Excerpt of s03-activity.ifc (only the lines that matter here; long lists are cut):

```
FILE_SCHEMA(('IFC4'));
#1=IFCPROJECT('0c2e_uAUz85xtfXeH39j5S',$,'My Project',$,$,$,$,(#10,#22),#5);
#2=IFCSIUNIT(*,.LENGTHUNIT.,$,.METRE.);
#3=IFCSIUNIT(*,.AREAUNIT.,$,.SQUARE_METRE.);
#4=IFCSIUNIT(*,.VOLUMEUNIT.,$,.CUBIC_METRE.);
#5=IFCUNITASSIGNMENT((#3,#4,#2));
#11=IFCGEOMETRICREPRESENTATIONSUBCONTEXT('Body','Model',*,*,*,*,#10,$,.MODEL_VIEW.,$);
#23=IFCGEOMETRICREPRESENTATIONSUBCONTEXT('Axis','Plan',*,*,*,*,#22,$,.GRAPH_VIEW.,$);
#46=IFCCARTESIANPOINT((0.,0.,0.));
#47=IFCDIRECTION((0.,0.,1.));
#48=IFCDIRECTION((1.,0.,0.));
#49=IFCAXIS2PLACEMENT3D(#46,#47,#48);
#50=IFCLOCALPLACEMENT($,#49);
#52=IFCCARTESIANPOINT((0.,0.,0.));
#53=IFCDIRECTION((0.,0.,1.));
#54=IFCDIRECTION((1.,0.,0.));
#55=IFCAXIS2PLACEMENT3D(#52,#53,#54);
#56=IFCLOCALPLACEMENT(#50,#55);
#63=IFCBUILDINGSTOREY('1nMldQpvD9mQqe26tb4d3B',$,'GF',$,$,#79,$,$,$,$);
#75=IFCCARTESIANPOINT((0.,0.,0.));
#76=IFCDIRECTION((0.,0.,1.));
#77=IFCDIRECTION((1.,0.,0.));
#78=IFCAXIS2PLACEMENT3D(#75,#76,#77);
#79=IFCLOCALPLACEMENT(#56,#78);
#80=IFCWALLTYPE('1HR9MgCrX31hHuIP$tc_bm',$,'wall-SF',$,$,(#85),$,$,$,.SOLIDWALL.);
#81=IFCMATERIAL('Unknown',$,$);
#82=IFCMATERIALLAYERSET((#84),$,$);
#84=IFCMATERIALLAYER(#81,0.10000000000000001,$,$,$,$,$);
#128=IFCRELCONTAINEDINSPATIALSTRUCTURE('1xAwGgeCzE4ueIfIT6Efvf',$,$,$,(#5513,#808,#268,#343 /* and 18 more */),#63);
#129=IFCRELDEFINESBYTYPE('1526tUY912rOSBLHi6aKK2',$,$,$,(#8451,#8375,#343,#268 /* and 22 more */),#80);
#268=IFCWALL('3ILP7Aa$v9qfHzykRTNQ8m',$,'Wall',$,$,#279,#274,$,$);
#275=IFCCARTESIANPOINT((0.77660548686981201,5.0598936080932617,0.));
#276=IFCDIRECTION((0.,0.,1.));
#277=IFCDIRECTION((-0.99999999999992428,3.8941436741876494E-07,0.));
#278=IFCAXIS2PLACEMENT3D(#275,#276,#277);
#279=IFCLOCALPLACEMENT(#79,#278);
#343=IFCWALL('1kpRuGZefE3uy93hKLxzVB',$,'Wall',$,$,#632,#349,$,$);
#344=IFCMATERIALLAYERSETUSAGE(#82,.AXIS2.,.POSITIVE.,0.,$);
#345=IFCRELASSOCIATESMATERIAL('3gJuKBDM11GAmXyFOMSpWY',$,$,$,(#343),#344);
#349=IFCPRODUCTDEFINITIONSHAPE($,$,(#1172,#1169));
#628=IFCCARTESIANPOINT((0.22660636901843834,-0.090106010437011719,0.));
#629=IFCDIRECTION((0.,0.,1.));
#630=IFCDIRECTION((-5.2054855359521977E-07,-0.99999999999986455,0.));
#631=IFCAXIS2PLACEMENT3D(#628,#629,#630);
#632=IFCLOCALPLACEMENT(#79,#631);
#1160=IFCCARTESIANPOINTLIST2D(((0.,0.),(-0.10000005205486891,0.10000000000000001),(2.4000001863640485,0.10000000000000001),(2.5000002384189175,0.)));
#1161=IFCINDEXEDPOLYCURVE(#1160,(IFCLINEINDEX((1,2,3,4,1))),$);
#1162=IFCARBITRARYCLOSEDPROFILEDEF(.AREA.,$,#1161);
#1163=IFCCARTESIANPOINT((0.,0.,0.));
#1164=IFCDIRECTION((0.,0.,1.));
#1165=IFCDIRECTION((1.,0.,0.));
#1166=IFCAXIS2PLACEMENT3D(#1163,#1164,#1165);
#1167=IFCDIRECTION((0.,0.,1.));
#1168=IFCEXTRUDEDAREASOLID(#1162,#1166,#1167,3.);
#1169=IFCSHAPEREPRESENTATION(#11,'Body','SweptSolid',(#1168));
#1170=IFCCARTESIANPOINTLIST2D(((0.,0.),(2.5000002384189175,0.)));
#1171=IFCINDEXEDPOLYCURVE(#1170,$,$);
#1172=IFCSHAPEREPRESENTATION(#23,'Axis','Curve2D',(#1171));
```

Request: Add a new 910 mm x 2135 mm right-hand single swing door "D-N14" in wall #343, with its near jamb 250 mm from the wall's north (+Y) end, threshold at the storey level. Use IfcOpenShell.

```python
import numpy as np
import ifcopenshell
import ifcopenshell.api.feature
import ifcopenshell.api.geometry
import ifcopenshell.api.root
import ifcopenshell.api.spatial
import ifcopenshell.geom
import ifcopenshell.util.element
import ifcopenshell.util.placement
import ifcopenshell.util.representation
import ifcopenshell.util.shape
import ifcopenshell.util.unit

model = ifcopenshell.open("s03-activity.ifc")
unit_scale = ifcopenshell.util.unit.calculate_unit_scale(model)
settings = ifcopenshell.geom.settings()


def volume(element):
    """Net volume in cubic metres, openings subtracted."""
    shape = ifcopenshell.geom.create_shape(settings, element)
    return ifcopenshell.util.shape.get_volume(shape.geometry)


wall = model.by_guid("1kpRuGZefE3uy93hKLxzVB")
storey = ifcopenshell.util.element.get_container(wall, ifc_class="IfcBuildingStorey")
context = ifcopenshell.util.representation.get_context(model, "Model", "Body", "MODEL_VIEW")
before = volume(wall)

width, height, from_end, sill = 0.91, 2.135, 0.25, 0.0  # metres

# The wall runs along its own X axis, and the end named is its -X end.
wall_shape = ifcopenshell.geom.create_shape(settings, wall)
x, y, z = ifcopenshell.util.shape.get_vertices(wall_shape.geometry).T
start = x.min() + from_end
face, thickness = float(y.min()), float(y.max() - y.min())
wall_matrix = ifcopenshell.util.placement.get_local_placement(wall.ObjectPlacement)
level = ifcopenshell.util.placement.get_local_placement(storey.ObjectPlacement)[2, 3]


def in_wall(x, y):
    """Placement at x, y metres in the wall's axes, at sill height."""
    matrix = wall_matrix.copy()
    matrix[:, 3] = wall_matrix @ np.array([x / unit_scale, y / unit_scale, 0.0, 1.0])
    matrix[2, 3] = level + sill / unit_scale
    return matrix


# Opening: a box that overshoots both wall faces by 50 mm.
opening = ifcopenshell.api.root.create_entity(model, ifc_class="IfcOpeningElement", predefined_type="OPENING")
box = ifcopenshell.api.geometry.add_wall_representation(
    model, context=context, length=width, height=height, thickness=thickness + 0.1
)
ifcopenshell.api.geometry.assign_representation(model, product=opening, representation=box)
ifcopenshell.api.geometry.edit_object_placement(model, product=opening, matrix=in_wall(start, face - 0.05), is_si=False)
ifcopenshell.api.feature.add_feature(model, feature=opening, element=wall)

door = ifcopenshell.api.root.create_entity(model, ifc_class="IfcDoor", name="D-N14", predefined_type="DOOR")
door.OverallWidth, door.OverallHeight = width / unit_scale, height / unit_scale
door.OperationType = "SINGLE_SWING_RIGHT"
body = ifcopenshell.api.geometry.add_door_representation(
    model,
    context=context,
    overall_width=door.OverallWidth,
    overall_height=door.OverallHeight,
    operation_type="SINGLE_SWING_RIGHT",
    lining_properties={"LiningDepth": thickness / unit_scale, "ThresholdDepth": thickness / unit_scale},
)
ifcopenshell.api.geometry.assign_representation(model, product=door, representation=body)
ifcopenshell.api.spatial.assign_container(model, products=[door], relating_structure=storey)
ifcopenshell.api.feature.add_filling(model, opening=opening, element=door)

# The lining spans the wall, so the door starts at the wall face.
ifcopenshell.api.geometry.edit_object_placement(model, product=door, matrix=in_wall(start, face), is_si=False)

after = volume(wall)

print(f"wall volume {before:.3f} -> {after:.3f} m3")

model.write("s03-activity_edited.ifc")
```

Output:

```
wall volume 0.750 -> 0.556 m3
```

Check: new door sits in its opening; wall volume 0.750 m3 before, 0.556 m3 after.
